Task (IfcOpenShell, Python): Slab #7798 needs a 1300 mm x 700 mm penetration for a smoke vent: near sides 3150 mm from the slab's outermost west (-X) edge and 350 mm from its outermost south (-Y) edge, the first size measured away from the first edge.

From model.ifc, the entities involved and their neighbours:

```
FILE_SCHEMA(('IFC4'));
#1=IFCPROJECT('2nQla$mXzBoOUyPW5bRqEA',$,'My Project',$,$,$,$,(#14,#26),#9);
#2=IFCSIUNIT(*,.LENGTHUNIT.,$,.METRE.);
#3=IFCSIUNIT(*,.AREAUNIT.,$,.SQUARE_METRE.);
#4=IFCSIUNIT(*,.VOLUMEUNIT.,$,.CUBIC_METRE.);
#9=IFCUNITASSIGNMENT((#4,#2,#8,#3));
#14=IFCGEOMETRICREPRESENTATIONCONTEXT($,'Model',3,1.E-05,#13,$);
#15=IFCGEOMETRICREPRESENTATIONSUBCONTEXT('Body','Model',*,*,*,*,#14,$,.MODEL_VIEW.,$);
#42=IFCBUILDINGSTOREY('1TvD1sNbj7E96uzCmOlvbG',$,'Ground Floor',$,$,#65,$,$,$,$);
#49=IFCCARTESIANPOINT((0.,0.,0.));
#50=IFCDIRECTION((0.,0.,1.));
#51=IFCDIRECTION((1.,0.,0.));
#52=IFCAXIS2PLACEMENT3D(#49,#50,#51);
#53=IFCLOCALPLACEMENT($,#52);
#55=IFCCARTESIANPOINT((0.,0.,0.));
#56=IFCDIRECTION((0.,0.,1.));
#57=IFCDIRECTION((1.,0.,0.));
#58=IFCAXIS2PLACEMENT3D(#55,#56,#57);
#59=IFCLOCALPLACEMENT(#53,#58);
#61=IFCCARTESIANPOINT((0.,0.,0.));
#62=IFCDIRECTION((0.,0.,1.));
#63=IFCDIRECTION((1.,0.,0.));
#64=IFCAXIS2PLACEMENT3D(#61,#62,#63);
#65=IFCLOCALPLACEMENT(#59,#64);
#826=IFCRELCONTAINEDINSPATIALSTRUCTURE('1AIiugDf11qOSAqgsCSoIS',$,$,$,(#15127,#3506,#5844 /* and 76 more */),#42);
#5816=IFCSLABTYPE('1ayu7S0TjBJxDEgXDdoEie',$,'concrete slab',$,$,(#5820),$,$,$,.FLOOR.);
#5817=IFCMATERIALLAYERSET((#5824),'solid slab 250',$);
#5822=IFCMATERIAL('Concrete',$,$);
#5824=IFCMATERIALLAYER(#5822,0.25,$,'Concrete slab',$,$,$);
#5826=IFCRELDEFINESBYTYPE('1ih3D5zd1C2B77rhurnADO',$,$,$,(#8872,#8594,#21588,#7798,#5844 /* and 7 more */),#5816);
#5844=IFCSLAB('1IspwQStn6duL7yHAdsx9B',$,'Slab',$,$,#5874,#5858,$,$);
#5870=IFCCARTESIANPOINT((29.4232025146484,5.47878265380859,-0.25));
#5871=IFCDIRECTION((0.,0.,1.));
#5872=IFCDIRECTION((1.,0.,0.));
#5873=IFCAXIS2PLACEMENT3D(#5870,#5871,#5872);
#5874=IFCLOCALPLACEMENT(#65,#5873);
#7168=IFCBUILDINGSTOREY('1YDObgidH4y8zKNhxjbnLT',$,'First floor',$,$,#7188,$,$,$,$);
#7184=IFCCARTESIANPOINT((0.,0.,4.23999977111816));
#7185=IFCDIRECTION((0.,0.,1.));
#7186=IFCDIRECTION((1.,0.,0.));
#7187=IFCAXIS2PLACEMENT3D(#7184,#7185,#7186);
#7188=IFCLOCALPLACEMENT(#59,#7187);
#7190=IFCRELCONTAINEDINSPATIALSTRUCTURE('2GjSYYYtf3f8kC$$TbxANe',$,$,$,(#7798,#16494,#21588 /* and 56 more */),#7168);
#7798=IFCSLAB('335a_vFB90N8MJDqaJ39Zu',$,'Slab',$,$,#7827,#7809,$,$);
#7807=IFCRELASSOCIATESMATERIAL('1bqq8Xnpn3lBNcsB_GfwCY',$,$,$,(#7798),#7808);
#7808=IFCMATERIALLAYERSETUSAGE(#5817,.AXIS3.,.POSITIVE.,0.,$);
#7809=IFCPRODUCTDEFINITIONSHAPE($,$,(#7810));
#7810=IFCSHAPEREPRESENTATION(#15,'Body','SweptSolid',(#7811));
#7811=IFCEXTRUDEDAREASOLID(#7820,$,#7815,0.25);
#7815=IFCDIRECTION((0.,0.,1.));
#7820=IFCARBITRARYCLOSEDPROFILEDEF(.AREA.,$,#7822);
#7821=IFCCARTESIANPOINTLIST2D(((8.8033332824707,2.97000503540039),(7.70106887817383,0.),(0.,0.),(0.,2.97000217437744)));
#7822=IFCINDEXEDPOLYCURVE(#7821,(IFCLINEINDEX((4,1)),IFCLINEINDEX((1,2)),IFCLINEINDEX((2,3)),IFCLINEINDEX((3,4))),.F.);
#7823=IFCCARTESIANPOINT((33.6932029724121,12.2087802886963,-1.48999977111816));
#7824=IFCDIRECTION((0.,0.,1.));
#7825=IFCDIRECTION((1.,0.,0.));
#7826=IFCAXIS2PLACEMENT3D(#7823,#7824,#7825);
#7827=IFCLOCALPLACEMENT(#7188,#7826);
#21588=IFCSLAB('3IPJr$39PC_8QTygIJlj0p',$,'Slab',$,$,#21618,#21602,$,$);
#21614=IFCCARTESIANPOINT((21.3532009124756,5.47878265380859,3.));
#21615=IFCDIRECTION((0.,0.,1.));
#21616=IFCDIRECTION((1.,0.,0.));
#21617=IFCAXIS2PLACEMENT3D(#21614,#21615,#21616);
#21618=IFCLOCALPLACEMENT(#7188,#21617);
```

```python
import numpy as np
import ifcopenshell
import ifcopenshell.api.feature
import ifcopenshell.api.geometry
import ifcopenshell.api.root
import ifcopenshell.geom
import ifcopenshell.util.placement
import ifcopenshell.util.representation
import ifcopenshell.util.shape
import ifcopenshell.util.unit

model = ifcopenshell.open("model.ifc")
unit_scale = ifcopenshell.util.unit.calculate_unit_scale(model)
settings = ifcopenshell.geom.settings()


def volume(element):
    """Net volume in cubic metres, openings subtracted."""
    shape = ifcopenshell.geom.create_shape(settings, element)
    return ifcopenshell.util.shape.get_volume(shape.geometry)


slab = model.by_guid("335a_vFB90N8MJDqaJ39Zu")
before = volume(slab)

# Extent in the slab's own axes, in metres. The edges named are its -X and -Y sides.
slab_shape = ifcopenshell.geom.create_shape(settings, slab)
vertices = ifcopenshell.util.shape.get_vertices(slab_shape.geometry)
x_min, y_min, bottom = vertices.min(axis=0)
top = vertices[:, 2].max()

opening = ifcopenshell.api.root.create_entity(model, ifc_class="IfcOpeningElement", name="Smoke vent opening", predefined_type="OPENING")
context = ifcopenshell.util.representation.get_context(model, "Model", "Body", "MODEL_VIEW")
width, depth = 1.3, 0.7
outline = [(0.0, 0.0), (width, 0.0), (width, depth), (0.0, depth), (0.0, 0.0)]
# Overshoot both faces by 50 mm so the cut is clean.
shape = ifcopenshell.api.geometry.add_slab_representation(
    model, context=context, depth=top - bottom + 0.1, polyline=outline
)
ifcopenshell.api.geometry.assign_representation(model, product=opening, representation=shape)

matrix = ifcopenshell.util.placement.get_local_placement(slab.ObjectPlacement)
matrix[:, 3] = matrix @ np.append(np.array([x_min + 3.15, y_min + 0.35, bottom - 0.05]) / unit_scale, 1.0)
ifcopenshell.api.geometry.edit_object_placement(model, product=opening, matrix=matrix, is_si=False)
ifcopenshell.api.feature.add_feature(model, feature=opening, element=slab)

after = volume(slab)

print(f"slab volume {before:.3f} -> {after:.3f} m3")

model.write("model_rev.ifc")
```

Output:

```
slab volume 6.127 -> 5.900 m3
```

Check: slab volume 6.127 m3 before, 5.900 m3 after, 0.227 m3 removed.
